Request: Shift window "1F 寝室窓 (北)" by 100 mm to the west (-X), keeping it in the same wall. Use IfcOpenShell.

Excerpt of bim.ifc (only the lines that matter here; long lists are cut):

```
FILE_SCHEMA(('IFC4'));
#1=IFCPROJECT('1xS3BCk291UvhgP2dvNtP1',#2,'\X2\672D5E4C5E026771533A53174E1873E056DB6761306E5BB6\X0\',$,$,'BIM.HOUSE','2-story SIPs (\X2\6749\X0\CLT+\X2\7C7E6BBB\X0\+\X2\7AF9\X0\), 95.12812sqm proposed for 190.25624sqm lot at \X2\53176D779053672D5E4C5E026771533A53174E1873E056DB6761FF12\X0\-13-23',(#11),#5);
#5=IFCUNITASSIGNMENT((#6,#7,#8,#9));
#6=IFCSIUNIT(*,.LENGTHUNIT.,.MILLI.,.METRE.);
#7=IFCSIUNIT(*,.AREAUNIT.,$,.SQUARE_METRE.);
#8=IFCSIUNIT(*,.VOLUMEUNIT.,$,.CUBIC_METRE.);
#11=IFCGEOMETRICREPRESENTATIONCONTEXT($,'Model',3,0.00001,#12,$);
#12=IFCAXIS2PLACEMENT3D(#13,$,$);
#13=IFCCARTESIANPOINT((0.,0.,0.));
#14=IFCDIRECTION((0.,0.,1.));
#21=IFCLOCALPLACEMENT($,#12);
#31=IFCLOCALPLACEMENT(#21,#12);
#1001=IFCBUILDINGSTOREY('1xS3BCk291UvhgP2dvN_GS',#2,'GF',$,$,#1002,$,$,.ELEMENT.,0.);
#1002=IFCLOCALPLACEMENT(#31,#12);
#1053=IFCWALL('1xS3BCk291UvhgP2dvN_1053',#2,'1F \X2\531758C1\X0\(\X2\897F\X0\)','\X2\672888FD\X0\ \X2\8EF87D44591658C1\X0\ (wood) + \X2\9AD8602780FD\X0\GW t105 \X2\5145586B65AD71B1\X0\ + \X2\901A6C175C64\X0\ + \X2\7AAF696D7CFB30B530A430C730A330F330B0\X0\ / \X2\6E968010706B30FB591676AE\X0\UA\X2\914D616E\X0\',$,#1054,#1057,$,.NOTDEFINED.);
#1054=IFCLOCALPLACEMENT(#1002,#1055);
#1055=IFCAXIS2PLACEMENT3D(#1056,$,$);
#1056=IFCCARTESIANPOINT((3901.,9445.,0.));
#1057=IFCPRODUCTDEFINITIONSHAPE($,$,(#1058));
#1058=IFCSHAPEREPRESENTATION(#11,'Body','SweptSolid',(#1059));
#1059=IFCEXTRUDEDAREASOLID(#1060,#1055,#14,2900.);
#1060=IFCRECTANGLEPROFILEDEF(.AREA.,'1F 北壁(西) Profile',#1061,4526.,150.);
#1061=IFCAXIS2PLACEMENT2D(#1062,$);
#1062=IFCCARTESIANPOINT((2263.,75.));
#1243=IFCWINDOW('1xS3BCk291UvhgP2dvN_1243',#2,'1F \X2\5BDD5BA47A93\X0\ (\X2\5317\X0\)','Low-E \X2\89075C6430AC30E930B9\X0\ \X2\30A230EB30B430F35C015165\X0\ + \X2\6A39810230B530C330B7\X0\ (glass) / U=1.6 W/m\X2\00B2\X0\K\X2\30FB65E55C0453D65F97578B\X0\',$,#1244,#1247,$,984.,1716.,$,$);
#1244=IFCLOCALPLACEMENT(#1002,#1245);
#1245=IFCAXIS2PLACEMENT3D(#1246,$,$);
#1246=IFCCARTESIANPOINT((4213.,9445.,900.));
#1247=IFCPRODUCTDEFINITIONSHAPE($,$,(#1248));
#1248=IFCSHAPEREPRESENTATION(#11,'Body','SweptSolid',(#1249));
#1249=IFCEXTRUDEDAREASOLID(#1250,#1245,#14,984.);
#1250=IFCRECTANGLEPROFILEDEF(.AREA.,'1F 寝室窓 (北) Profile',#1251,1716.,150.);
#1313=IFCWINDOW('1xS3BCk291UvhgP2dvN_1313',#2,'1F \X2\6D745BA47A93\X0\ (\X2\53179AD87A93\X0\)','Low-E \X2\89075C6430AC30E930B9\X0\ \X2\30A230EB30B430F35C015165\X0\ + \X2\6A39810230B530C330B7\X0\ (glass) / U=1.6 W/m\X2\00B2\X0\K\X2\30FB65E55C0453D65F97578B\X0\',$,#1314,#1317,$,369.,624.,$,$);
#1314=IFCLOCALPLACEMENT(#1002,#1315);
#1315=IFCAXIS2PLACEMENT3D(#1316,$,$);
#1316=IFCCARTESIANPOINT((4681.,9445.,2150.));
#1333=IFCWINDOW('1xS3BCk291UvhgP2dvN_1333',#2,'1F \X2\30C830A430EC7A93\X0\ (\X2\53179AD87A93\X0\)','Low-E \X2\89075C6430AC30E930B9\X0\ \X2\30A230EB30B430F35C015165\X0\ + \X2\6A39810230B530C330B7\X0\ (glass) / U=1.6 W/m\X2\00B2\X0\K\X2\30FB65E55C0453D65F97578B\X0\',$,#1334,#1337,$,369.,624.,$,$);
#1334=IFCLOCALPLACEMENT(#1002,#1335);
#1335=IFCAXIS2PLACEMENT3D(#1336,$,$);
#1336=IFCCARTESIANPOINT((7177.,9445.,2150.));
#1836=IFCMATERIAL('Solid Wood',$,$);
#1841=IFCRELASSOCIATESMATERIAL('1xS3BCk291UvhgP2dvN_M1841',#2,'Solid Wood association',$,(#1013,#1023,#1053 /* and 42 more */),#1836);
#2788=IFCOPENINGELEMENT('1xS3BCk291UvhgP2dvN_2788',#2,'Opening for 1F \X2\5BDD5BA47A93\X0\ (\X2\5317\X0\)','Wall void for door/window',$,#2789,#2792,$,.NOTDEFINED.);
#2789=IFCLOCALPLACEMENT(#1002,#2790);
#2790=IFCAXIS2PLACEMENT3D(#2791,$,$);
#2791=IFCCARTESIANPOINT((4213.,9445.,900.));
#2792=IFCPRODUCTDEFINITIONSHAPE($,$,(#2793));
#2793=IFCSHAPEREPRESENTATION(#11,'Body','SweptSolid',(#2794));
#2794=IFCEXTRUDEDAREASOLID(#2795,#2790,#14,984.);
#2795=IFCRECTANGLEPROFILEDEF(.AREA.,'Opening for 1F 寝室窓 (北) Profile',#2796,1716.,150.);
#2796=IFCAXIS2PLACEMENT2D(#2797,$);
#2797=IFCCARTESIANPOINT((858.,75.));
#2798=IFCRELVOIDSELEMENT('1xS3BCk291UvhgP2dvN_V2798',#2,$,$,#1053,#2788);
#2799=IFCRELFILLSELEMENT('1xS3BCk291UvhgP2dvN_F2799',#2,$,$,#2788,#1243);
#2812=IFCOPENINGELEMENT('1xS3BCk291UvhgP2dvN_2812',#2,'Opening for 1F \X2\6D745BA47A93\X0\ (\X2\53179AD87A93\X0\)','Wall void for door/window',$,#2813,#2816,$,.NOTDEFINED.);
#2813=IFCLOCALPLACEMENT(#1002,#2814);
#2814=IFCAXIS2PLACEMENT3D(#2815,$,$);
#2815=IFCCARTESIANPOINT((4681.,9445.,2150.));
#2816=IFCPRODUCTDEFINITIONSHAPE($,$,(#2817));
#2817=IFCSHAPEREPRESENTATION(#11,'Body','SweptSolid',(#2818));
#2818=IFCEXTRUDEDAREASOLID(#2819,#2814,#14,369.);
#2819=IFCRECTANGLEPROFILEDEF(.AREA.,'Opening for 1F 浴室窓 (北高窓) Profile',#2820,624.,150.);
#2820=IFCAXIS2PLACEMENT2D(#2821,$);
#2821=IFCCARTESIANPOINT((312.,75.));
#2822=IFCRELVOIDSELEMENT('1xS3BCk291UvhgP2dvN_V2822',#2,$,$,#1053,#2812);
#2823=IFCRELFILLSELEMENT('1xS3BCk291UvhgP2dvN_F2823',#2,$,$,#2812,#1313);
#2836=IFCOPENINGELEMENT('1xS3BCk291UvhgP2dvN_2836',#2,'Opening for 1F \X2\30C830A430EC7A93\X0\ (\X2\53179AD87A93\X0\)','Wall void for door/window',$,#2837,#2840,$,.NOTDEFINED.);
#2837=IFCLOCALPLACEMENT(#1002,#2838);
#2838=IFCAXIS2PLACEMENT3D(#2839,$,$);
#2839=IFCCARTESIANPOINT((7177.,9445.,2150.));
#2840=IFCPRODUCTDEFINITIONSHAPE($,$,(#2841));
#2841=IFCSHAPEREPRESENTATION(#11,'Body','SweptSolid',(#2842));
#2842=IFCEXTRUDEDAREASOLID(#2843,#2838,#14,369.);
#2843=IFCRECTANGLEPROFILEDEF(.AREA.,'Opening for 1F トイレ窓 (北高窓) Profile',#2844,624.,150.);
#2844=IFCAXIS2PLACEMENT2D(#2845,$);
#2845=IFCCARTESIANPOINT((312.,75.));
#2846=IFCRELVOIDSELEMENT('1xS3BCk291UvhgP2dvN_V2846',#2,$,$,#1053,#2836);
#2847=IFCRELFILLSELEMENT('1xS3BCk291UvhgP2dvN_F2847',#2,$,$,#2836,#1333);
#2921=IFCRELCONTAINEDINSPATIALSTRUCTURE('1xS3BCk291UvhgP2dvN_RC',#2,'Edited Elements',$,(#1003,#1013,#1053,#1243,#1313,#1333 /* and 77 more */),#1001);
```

```python
import ifcopenshell
import ifcopenshell.api.geometry
import ifcopenshell.util.placement
import ifcopenshell.util.unit

model = ifcopenshell.open("bim.ifc")
unit_scale = ifcopenshell.util.unit.calculate_unit_scale(model)

window = model.by_guid("1xS3BCk291UvhgP2dvN_1243")
opening = window.FillsVoids[0].RelatingOpeningElement
wall = opening.VoidsElements[0].RelatingBuildingElement

wall_matrix = ifcopenshell.util.placement.get_local_placement(wall.ObjectPlacement)
shift = wall_matrix[:3, 0] * -0.1 / unit_scale
before = ifcopenshell.util.placement.get_local_placement(window.ObjectPlacement)[:3, 3].copy()

# The window is not placed relative to its opening, so move both.
for product in (opening, window):
    matrix = ifcopenshell.util.placement.get_local_placement(product.ObjectPlacement)
    matrix[:3, 3] += shift
    ifcopenshell.api.geometry.edit_object_placement(model, product=product, matrix=matrix, is_si=False)

after = ifcopenshell.util.placement.get_local_placement(window.ObjectPlacement)[:3, 3]
print("window moved by", (after - before).round(3) + 0.0)

model.write("bim-out.ifc")
```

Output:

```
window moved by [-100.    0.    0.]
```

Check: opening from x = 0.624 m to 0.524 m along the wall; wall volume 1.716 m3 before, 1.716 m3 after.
